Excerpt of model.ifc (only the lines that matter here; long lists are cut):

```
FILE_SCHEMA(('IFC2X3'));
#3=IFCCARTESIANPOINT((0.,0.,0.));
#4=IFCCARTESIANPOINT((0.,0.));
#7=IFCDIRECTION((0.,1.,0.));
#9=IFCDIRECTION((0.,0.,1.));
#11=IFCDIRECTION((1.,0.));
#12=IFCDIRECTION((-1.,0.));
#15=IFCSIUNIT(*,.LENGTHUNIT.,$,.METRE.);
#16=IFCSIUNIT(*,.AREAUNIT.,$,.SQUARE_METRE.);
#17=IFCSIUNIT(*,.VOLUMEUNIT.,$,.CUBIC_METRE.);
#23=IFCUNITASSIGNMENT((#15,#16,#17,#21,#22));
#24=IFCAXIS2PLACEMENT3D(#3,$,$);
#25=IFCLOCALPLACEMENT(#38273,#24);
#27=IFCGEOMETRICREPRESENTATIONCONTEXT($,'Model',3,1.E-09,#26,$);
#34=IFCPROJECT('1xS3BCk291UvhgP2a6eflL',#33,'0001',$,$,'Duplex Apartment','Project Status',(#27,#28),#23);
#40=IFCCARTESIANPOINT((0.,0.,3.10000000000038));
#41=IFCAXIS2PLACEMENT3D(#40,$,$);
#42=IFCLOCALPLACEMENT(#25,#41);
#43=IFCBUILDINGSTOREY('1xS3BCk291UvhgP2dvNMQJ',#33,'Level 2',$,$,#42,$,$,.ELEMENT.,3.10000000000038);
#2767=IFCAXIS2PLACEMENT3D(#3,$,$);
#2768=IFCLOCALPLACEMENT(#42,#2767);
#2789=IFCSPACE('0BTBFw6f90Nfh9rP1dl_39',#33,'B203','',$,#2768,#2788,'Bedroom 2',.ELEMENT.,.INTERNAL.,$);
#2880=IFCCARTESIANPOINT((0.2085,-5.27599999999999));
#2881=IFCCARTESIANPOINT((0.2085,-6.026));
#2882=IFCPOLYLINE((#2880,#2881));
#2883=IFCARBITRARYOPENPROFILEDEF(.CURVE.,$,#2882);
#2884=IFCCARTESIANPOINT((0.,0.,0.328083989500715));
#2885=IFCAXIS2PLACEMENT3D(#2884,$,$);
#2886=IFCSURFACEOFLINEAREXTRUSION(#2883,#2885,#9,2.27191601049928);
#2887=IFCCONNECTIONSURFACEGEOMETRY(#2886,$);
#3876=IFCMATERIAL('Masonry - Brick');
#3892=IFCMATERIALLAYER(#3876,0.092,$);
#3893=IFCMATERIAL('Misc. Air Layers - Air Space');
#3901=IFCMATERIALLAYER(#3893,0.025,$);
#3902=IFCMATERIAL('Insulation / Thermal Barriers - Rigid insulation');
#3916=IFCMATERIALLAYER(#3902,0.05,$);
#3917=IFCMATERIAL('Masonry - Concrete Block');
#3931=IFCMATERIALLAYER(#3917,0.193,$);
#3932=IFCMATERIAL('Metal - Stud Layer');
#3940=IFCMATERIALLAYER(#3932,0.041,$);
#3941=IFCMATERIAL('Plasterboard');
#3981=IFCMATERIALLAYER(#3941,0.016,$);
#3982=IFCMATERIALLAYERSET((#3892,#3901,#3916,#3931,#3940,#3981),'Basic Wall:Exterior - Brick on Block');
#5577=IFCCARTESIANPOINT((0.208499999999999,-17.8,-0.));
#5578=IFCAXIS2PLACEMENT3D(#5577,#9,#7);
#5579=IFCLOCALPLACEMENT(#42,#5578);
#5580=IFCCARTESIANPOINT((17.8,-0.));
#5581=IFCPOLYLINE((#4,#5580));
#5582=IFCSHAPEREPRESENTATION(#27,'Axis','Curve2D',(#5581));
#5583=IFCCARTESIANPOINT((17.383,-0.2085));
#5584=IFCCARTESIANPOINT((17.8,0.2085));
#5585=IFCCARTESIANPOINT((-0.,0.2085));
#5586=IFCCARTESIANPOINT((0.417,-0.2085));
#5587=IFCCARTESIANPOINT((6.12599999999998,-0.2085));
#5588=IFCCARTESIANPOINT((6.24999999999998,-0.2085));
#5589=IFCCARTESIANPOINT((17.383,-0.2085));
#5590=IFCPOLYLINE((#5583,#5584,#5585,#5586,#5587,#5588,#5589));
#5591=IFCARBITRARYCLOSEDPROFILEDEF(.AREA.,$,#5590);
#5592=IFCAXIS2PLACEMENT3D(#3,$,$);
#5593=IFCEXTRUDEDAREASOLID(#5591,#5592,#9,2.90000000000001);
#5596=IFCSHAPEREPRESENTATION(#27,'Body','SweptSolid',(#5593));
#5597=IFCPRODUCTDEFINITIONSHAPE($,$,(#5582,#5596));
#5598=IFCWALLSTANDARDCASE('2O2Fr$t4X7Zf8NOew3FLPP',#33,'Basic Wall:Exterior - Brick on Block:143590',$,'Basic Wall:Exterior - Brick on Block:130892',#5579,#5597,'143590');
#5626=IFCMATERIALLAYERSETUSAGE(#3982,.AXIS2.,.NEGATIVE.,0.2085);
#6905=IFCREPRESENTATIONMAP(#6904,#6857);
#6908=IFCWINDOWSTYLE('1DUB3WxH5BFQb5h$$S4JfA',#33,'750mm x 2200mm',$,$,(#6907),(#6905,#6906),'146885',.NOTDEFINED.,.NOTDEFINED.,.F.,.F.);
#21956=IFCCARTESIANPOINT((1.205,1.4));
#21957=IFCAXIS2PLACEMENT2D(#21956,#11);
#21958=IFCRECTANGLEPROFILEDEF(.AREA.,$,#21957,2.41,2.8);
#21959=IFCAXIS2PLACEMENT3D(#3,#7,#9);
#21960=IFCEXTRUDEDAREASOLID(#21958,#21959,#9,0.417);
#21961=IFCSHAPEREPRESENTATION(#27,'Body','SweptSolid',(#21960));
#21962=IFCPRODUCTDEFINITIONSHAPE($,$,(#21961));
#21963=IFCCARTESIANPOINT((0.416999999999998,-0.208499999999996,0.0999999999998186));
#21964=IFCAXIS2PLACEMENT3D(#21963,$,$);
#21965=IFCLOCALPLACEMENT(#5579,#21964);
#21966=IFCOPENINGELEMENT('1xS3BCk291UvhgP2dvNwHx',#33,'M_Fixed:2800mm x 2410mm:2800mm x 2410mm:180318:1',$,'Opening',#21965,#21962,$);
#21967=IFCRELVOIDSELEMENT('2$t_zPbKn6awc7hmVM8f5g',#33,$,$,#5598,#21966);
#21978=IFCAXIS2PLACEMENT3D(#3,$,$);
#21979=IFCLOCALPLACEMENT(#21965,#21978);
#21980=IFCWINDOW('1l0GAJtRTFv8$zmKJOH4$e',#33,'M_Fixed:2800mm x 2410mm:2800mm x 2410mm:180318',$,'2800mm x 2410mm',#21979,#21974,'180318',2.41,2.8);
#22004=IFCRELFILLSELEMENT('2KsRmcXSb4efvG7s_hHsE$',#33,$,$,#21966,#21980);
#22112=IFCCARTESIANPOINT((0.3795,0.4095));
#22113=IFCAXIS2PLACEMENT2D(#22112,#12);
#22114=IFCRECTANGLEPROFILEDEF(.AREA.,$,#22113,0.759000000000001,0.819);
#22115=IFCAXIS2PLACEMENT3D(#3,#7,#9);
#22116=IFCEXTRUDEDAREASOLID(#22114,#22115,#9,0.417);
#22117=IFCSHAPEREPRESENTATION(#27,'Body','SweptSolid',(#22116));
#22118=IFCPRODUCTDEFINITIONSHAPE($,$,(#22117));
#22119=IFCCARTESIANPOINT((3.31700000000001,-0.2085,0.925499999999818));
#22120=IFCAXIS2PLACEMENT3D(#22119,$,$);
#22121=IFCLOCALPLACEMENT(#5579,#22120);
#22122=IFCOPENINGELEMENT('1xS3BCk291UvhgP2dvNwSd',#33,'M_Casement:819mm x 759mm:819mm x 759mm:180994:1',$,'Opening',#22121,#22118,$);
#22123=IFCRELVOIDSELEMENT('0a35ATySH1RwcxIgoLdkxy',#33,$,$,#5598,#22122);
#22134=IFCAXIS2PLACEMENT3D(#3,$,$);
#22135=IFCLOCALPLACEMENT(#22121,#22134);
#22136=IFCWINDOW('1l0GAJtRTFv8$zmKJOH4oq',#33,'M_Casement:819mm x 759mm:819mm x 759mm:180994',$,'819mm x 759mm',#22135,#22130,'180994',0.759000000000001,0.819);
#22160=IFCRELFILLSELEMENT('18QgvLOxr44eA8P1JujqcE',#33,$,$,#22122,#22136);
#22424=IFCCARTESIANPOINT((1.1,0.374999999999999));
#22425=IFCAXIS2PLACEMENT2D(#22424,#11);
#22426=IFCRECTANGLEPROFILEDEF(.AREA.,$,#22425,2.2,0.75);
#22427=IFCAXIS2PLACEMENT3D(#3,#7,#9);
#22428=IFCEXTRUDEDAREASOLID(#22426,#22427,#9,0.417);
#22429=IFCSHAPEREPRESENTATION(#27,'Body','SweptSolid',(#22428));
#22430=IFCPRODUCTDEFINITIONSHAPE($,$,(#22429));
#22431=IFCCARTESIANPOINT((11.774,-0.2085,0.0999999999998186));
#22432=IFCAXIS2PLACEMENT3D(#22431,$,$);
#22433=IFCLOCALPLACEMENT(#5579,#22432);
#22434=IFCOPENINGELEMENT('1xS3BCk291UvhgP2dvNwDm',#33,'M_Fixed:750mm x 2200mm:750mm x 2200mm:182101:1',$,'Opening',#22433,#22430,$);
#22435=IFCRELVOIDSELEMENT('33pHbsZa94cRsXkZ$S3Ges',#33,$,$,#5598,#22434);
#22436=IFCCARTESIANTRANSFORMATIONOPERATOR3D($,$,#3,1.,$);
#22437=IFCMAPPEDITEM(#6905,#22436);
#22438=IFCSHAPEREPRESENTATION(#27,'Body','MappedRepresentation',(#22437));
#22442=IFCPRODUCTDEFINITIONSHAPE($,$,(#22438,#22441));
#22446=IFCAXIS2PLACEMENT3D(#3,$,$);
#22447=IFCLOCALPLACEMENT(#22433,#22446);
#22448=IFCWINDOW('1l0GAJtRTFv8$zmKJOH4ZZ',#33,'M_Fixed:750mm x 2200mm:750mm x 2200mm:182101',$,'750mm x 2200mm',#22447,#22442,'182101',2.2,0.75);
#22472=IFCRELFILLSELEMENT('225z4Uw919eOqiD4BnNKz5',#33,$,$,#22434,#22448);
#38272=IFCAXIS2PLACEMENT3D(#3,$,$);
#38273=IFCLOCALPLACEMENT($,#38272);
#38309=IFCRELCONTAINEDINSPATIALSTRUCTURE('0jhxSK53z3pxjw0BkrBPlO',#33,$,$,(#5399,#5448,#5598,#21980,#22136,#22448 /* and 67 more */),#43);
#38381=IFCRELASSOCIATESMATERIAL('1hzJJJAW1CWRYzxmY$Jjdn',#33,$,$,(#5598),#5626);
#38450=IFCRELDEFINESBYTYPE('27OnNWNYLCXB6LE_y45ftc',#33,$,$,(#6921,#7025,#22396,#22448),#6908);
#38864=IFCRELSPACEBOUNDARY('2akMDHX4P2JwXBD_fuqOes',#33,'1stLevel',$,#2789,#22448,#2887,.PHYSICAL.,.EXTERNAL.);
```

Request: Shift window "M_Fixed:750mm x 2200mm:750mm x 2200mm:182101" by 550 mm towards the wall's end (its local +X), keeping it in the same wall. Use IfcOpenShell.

```python
import numpy as np
import ifcopenshell
import ifcopenshell.api.geometry
import ifcopenshell.util.placement

model = ifcopenshell.open("model.ifc")

window = model.by_id(22448)
opening = window.FillsVoids[0].RelatingOpeningElement
wall = opening.VoidsElements[0].RelatingBuildingElement

wall_matrix = ifcopenshell.util.placement.get_local_placement(wall.ObjectPlacement)
shift = wall_matrix[:3, 0] * 0.55
before = ifcopenshell.util.placement.get_local_placement(window.ObjectPlacement)[:3, 3].copy()

# The window is placed relative to its opening, so it follows when the opening moves.
matrix = ifcopenshell.util.placement.get_local_placement(opening.ObjectPlacement)
matrix[:3, 3] += shift
ifcopenshell.api.geometry.edit_object_placement(
    model, product=opening, matrix=matrix, is_si=False, should_transform_children=True
)

# Space boundary surfaces are stored in each space's coordinates; move them too.
for rel in window.ProvidesBoundaries:
    if not rel.ConnectionGeometry:
        continue
    surface = rel.ConnectionGeometry.SurfaceOnRelatingElement
    space_matrix = ifcopenshell.util.placement.get_local_placement(rel.RelatingSpace.ObjectPlacement)
    point = np.array(surface.Position.Location.Coordinates) + space_matrix[:3, :3].T @ shift
    surface.Position = model.createIfcAxis2Placement3D(
        model.createIfcCartesianPoint(point.tolist()), surface.Position.Axis, surface.Position.RefDirection
    )

after = ifcopenshell.util.placement.get_local_placement(window.ObjectPlacement)[:3, 3]
print("window moved by", (after - before).round(3) + 0.0)

model.write("model_edited.ifc")
```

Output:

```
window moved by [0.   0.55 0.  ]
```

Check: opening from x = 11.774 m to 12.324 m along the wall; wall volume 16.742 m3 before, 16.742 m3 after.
